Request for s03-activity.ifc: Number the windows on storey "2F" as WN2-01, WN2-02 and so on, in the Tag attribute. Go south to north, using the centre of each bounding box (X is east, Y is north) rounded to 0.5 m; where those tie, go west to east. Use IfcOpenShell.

First a look at what the model holds.

```python
import ifcopenshell
import ifcopenshell.util.element
import ifcopenshell.util.placement

model = ifcopenshell.open("s03-activity.ifc")
print(model.schema)
storey = next(s for s in model.by_type("IfcBuildingStorey") if s.Name == "2F")
windows = [e for e in ifcopenshell.util.element.get_decomposition(storey) if e.is_a("IfcWindow")]
for e in sorted(windows, key=lambda e: e.id()):
    origin = ifcopenshell.util.placement.get_local_placement(e.ObjectPlacement)[:3, 3]
    print(e.id(), e.Tag, e.Name, origin.round(2) + 0.0, sep=" | ")
```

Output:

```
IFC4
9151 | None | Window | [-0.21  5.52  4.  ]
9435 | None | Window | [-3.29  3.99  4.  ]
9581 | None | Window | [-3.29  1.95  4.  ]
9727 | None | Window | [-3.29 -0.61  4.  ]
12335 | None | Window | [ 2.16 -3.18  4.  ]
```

```python
import ifcopenshell
import ifcopenshell.geom
import ifcopenshell.util.element
import ifcopenshell.util.shape

model = ifcopenshell.open("s03-activity.ifc")
settings = ifcopenshell.geom.settings()
settings.set("use-world-coords", True)


def centre(element):
    shape = ifcopenshell.geom.create_shape(settings, element)
    return ifcopenshell.util.shape.get_bbox_centroid(shape.geometry)


storey = next(s for s in model.by_type("IfcBuildingStorey") if s.Name == "2F")
windows = [e for e in ifcopenshell.util.element.get_decomposition(storey) if e.is_a("IfcWindow")]

# Insertion points can sit at a corner or the storey origin, so sort by the geometry (in metres).
centres = {e: centre(e) for e in windows}
windows.sort(key=lambda e: (round(centres[e][1] / 0.5), centres[e][0]))

for i, e in enumerate(windows, start=1):
    number = f"WN2-{i:02d}"
    e.Tag = number
    print(e.id(), number)

model.write("s03-activity_rev.ifc")
```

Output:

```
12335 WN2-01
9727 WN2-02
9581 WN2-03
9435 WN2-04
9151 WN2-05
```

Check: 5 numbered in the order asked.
